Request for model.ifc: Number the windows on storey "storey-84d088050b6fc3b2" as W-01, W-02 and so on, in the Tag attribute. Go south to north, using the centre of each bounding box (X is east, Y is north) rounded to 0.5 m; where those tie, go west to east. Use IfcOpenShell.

First a look at what the model holds.

```python
import ifcopenshell
import ifcopenshell.util.element
import ifcopenshell.util.placement

model = ifcopenshell.open("model.ifc")
print(model.schema)
storey = next(s for s in model.by_type("IfcBuildingStorey") if s.Name == "storey-84d088050b6fc3b2")
windows = [e for e in ifcopenshell.util.element.get_decomposition(storey) if e.is_a("IfcWindow")]
for e in sorted(windows, key=lambda e: e.id()):
    origin = ifcopenshell.util.placement.get_local_placement(e.ObjectPlacement)[:3, 3]
    print(e.id(), e.Tag, e.Name, origin.round(2) + 0.0, sep=" | ")
```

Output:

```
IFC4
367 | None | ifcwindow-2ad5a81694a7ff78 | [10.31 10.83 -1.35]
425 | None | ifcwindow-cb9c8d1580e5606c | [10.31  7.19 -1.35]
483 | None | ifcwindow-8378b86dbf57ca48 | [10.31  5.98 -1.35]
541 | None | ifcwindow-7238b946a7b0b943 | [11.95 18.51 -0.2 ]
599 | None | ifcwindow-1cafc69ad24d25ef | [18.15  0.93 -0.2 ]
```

```python
import ifcopenshell
import ifcopenshell.geom
import ifcopenshell.util.element
import ifcopenshell.util.shape

model = ifcopenshell.open("model.ifc")
settings = ifcopenshell.geom.settings()
settings.set("use-world-coords", True)


def centre(element):
    shape = ifcopenshell.geom.create_shape(settings, element)
    return ifcopenshell.util.shape.get_bbox_centroid(shape.geometry)


storey = next(s for s in model.by_type("IfcBuildingStorey") if s.Name == "storey-84d088050b6fc3b2")
windows = [e for e in ifcopenshell.util.element.get_decomposition(storey) if e.is_a("IfcWindow")]

# Insertion points can sit at a corner or the storey origin, so sort by the geometry (in metres).
centres = {e: centre(e) for e in windows}
windows.sort(key=lambda e: (round(centres[e][1] / 0.5), centres[e][0]))

for i, e in enumerate(windows, start=1):
    number = f"W-{i:02d}"
    e.Tag = number
    print(e.id(), number)

model.write("model_v2.ifc")
```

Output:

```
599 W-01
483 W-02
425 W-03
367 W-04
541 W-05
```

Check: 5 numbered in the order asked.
